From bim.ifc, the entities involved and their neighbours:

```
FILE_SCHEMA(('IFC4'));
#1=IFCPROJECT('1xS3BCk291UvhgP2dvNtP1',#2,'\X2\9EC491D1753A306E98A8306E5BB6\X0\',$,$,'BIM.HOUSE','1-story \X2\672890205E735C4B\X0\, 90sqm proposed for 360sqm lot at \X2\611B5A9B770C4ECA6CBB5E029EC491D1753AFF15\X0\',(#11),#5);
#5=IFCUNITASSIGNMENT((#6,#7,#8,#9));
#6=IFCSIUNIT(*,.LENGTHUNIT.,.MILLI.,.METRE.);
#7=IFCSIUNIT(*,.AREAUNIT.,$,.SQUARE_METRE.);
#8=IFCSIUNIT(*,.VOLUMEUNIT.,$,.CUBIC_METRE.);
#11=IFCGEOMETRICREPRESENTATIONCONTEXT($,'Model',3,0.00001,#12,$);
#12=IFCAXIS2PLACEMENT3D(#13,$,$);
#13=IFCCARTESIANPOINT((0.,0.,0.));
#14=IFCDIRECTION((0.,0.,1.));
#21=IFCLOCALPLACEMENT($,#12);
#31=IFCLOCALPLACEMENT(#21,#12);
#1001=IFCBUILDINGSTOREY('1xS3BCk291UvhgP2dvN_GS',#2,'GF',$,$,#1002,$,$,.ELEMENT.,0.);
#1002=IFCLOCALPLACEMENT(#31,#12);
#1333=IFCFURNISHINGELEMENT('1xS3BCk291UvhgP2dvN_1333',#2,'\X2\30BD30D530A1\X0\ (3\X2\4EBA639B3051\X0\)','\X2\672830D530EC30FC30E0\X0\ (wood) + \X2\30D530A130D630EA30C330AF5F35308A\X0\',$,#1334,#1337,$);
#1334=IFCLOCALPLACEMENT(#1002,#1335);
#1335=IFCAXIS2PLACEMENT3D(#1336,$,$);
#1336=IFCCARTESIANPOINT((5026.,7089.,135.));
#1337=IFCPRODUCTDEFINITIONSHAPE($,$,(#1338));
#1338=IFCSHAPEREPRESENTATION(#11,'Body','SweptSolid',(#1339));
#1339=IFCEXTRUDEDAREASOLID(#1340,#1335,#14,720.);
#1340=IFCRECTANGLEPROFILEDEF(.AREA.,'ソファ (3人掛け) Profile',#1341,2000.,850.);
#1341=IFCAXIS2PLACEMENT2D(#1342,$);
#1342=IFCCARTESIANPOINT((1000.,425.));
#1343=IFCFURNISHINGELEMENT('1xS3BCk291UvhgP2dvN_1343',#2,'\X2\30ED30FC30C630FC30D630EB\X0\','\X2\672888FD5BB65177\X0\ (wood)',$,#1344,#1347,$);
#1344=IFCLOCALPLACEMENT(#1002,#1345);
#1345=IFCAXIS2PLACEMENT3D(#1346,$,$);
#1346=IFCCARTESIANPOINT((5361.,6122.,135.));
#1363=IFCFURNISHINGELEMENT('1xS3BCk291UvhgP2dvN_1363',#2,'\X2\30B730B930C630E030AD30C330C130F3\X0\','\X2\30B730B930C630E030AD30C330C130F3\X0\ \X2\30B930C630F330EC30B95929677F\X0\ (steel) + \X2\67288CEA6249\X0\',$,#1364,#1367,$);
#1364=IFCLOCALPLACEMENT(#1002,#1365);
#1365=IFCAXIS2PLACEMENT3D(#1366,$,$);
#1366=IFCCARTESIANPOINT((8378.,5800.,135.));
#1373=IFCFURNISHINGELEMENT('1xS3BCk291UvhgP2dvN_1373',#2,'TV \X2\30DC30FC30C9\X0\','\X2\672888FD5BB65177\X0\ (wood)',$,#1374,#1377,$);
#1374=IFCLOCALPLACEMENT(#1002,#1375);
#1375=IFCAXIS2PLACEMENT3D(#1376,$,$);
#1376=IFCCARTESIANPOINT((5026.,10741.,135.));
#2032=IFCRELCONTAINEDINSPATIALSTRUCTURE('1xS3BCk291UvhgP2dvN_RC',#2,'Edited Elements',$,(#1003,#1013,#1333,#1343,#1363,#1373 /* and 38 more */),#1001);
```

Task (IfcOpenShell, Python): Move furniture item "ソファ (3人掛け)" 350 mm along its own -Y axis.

```python
import ifcopenshell
import ifcopenshell.api.geometry
import ifcopenshell.util.placement

model = ifcopenshell.open("bim.ifc")

item = model.by_guid("1xS3BCk291UvhgP2dvN_1333")
matrix = ifcopenshell.util.placement.get_local_placement(item.ObjectPlacement)
matrix[:3, 3] -= matrix[:3, 1] * 350.0
ifcopenshell.api.geometry.edit_object_placement(model, product=item, matrix=matrix, is_si=False)

print(ifcopenshell.util.placement.get_local_placement(item.ObjectPlacement).round(3) + 0.0)

model.write("bim-out.ifc")
```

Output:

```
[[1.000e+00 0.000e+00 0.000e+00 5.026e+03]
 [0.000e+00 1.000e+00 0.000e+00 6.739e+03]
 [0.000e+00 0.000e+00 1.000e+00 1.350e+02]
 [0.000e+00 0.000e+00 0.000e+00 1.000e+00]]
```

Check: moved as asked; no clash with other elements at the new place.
